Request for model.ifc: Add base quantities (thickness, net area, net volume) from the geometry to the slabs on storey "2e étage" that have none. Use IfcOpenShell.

First a look at what the model holds.

```python
import ifcopenshell
import ifcopenshell.util.element
import ifcopenshell.util.unit

model = ifcopenshell.open("model.ifc")
print(model.schema)
for unit_type in ("LENGTHUNIT", "AREAUNIT", "VOLUMEUNIT"):
    print(unit_type, ifcopenshell.util.unit.calculate_unit_scale(model, unit_type))
storey = next(s for s in model.by_type("IfcBuildingStorey") if s.Name == "2e étage")
slabs = [e for e in ifcopenshell.util.element.get_decomposition(storey) if e.is_a("IfcSlab")]
for e in sorted(slabs, key=lambda e: e.id()):
    print(e.id(), e.is_a(), e.Name, list(ifcopenshell.util.element.get_psets(e, qtos_only=True)), sep=" | ")
```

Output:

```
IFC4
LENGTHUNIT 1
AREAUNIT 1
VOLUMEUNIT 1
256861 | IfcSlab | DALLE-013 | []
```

```python
import ifcopenshell
import ifcopenshell.api.pset
import ifcopenshell.geom
import ifcopenshell.util.element
import ifcopenshell.util.shape
import ifcopenshell.util.unit

model = ifcopenshell.open("model.ifc")
unit_scale = ifcopenshell.util.unit.calculate_unit_scale(model)
area_scale = ifcopenshell.util.unit.calculate_unit_scale(model, "AREAUNIT")
volume_scale = ifcopenshell.util.unit.calculate_unit_scale(model, "VOLUMEUNIT")
settings = ifcopenshell.geom.settings()

storey = next(s for s in model.by_type("IfcBuildingStorey") if s.Name == "2e étage")
slabs = [e for e in ifcopenshell.util.element.get_decomposition(storey) if e.is_a("IfcSlab")]

for e in sorted(slabs, key=lambda e: e.id()):
    if ifcopenshell.util.element.get_psets(e, qtos_only=True, should_inherit=False):
        continue
    # Geometry comes back in metres, in the element's own axes.
    shape = ifcopenshell.geom.create_shape(settings, e)
    values = {
        "Width": ifcopenshell.util.shape.get_z(shape.geometry) / unit_scale,
        "NetArea": ifcopenshell.util.shape.get_footprint_area(shape.geometry) / area_scale,
        "NetVolume": ifcopenshell.util.shape.get_volume(shape.geometry) / volume_scale,
    }
    qto = ifcopenshell.api.pset.add_qto(model, product=e, name="Qto_SlabBaseQuantities")
    ifcopenshell.api.pset.edit_qto(model, qto=qto, properties=values)
    print(e.id(), {k: round(v, 3) for k, v in values.items()})

model.write("model_rev.ifc")
```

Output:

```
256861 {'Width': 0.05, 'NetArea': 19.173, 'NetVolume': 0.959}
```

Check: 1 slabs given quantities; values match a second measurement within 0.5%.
